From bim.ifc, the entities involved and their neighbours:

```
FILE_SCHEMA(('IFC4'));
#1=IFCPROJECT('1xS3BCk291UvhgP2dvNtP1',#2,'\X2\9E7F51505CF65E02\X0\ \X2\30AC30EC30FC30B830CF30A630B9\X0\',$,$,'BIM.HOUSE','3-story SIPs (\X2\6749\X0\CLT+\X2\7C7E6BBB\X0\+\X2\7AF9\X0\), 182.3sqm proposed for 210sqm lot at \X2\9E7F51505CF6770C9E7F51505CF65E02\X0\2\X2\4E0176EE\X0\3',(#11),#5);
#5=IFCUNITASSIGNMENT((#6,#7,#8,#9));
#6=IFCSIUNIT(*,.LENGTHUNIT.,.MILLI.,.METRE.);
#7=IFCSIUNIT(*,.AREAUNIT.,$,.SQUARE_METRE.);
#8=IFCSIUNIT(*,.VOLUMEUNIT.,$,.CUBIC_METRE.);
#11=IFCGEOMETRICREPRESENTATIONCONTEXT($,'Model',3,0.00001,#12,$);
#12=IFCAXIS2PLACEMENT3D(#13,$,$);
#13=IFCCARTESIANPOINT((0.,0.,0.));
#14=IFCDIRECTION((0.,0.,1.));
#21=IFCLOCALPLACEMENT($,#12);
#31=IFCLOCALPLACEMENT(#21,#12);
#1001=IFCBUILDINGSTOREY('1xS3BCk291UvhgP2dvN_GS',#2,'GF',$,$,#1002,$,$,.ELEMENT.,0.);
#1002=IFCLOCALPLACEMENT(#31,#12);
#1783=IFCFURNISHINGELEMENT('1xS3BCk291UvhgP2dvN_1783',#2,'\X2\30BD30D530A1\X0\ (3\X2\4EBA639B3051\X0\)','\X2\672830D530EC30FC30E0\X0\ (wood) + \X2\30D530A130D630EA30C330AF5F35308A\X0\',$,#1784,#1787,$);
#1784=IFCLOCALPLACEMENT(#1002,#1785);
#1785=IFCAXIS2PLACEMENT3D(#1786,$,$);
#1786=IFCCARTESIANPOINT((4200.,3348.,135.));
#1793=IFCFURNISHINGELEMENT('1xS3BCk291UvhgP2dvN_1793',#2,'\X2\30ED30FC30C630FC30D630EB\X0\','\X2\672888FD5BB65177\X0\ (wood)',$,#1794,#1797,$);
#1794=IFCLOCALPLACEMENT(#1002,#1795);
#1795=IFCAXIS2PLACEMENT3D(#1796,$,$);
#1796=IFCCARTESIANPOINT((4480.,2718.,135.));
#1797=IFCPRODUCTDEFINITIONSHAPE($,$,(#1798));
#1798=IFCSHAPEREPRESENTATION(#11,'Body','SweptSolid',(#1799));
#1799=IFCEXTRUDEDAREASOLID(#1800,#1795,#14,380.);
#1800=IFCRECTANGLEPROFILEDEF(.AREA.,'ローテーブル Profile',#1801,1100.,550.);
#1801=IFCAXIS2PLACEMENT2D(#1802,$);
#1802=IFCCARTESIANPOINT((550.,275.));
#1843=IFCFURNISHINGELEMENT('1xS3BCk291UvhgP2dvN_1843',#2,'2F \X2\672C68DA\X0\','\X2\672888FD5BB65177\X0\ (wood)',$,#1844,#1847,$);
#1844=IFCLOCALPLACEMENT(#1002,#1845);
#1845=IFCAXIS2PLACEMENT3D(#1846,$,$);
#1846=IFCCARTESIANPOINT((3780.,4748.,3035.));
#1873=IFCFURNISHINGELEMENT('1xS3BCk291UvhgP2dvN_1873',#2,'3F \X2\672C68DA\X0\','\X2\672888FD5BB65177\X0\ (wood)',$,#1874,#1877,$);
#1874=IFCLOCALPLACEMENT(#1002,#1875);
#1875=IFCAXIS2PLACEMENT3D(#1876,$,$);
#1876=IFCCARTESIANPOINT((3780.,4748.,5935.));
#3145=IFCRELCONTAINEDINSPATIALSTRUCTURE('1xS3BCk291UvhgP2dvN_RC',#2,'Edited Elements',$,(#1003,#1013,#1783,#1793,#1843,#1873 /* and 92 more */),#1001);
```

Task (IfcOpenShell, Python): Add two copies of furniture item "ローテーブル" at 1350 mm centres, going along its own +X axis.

```python
import ifcopenshell
import ifcopenshell.api.geometry
import ifcopenshell.api.root
import ifcopenshell.util.element
import ifcopenshell.util.placement
import ifcopenshell.util.unit

model = ifcopenshell.open("bim.ifc")
unit_scale = ifcopenshell.util.unit.calculate_unit_scale(model)


def reuse_history(source, copy):
    """copy_class also copies each property set's owner history, people and application; keep the originals."""
    for rel in copy.IsDefinedBy:
        if rel.is_a("IfcRelDefinesByProperties") and (history := rel.RelatingPropertyDefinition.OwnerHistory):
            rel.RelatingPropertyDefinition.OwnerHistory = source.OwnerHistory
            ifcopenshell.util.element.remove_deep2(model, history)


source = model.by_id(1793)
base = ifcopenshell.util.placement.get_local_placement(source.ObjectPlacement)
step = base[:3, 0] * 1.35 / unit_scale

for i in range(1, 3):
    copy = ifcopenshell.api.root.copy_class(model, product=source)
    copy.Representation = ifcopenshell.util.element.copy_deep(
        model, source.Representation, exclude=["IfcGeometricRepresentationContext", "IfcRepresentationMap"]
    )
    reuse_history(source, copy)
    matrix = base.copy()
    matrix[:3, 3] += i * step
    print("added at", matrix[:3, 3].round(3) + 0.0)
    ifcopenshell.api.geometry.edit_object_placement(model, product=copy, matrix=matrix, is_si=False)

model.write("bim_edited.ifc")
```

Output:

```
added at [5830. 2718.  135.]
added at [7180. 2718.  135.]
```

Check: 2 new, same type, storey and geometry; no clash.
